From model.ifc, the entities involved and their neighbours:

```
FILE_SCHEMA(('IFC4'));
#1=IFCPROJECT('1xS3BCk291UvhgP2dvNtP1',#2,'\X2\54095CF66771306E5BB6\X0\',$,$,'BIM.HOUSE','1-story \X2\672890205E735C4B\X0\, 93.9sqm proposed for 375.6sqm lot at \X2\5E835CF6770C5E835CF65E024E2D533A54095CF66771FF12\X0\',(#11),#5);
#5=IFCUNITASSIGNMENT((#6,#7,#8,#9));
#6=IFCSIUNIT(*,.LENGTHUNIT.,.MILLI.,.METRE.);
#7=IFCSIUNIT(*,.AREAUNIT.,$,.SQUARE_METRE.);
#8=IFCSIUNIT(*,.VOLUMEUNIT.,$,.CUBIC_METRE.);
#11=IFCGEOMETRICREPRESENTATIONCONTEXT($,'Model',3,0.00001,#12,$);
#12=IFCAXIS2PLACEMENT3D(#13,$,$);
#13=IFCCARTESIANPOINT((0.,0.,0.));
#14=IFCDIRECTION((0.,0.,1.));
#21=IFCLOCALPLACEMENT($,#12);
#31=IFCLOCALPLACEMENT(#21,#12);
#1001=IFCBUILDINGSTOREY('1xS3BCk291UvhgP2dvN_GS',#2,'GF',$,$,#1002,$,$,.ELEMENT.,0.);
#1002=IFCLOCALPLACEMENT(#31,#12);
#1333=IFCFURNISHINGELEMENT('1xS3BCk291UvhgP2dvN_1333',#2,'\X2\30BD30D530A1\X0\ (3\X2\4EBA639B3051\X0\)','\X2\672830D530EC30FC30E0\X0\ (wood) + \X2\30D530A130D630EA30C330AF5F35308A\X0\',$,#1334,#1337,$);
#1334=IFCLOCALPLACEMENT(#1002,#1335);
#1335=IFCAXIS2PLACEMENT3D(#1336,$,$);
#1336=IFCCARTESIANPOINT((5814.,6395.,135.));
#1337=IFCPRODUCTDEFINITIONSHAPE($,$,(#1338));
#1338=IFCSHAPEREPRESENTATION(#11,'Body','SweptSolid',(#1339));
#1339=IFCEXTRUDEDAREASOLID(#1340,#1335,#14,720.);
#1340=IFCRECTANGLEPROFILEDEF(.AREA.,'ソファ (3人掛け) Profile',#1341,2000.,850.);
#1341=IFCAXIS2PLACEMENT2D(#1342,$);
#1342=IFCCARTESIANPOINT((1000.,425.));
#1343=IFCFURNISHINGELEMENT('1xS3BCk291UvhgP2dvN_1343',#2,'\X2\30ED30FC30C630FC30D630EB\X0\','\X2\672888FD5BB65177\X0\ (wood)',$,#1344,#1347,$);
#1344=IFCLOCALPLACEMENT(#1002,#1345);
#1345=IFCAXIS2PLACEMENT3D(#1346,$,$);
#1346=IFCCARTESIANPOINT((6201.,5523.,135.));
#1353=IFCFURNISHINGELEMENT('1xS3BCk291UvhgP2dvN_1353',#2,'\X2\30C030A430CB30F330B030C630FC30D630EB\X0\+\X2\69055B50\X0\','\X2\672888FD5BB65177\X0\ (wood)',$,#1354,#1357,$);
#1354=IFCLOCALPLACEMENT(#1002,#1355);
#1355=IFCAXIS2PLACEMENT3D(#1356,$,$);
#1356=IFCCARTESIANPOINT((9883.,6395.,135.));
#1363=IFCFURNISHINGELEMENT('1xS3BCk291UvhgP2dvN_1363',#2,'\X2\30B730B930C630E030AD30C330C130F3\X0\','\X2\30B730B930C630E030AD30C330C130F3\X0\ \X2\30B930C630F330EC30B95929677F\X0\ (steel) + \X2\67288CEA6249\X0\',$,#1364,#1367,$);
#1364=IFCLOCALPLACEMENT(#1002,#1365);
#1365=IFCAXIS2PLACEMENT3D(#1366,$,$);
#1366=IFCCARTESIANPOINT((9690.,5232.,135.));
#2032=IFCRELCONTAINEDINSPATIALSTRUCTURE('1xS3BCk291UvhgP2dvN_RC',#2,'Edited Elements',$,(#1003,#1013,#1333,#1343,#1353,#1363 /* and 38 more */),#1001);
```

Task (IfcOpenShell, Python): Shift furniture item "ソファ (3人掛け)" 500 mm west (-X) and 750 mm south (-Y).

```python
import ifcopenshell
import ifcopenshell.api.geometry
import ifcopenshell.util.placement
import ifcopenshell.util.unit

model = ifcopenshell.open("model.ifc")
unit_scale = ifcopenshell.util.unit.calculate_unit_scale(model)

item = model.by_id(1333)
matrix = ifcopenshell.util.placement.get_local_placement(item.ObjectPlacement)
matrix[0, 3] -= 0.5 / unit_scale
matrix[1, 3] -= 0.75 / unit_scale
ifcopenshell.api.geometry.edit_object_placement(model, product=item, matrix=matrix, is_si=False)

print(ifcopenshell.util.placement.get_local_placement(item.ObjectPlacement).round(3) + 0.0)

model.write("model_updated.ifc")
```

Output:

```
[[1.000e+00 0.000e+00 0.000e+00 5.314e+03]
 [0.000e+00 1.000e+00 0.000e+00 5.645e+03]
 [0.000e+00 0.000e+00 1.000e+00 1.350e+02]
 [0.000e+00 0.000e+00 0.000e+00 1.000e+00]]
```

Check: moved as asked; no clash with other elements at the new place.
